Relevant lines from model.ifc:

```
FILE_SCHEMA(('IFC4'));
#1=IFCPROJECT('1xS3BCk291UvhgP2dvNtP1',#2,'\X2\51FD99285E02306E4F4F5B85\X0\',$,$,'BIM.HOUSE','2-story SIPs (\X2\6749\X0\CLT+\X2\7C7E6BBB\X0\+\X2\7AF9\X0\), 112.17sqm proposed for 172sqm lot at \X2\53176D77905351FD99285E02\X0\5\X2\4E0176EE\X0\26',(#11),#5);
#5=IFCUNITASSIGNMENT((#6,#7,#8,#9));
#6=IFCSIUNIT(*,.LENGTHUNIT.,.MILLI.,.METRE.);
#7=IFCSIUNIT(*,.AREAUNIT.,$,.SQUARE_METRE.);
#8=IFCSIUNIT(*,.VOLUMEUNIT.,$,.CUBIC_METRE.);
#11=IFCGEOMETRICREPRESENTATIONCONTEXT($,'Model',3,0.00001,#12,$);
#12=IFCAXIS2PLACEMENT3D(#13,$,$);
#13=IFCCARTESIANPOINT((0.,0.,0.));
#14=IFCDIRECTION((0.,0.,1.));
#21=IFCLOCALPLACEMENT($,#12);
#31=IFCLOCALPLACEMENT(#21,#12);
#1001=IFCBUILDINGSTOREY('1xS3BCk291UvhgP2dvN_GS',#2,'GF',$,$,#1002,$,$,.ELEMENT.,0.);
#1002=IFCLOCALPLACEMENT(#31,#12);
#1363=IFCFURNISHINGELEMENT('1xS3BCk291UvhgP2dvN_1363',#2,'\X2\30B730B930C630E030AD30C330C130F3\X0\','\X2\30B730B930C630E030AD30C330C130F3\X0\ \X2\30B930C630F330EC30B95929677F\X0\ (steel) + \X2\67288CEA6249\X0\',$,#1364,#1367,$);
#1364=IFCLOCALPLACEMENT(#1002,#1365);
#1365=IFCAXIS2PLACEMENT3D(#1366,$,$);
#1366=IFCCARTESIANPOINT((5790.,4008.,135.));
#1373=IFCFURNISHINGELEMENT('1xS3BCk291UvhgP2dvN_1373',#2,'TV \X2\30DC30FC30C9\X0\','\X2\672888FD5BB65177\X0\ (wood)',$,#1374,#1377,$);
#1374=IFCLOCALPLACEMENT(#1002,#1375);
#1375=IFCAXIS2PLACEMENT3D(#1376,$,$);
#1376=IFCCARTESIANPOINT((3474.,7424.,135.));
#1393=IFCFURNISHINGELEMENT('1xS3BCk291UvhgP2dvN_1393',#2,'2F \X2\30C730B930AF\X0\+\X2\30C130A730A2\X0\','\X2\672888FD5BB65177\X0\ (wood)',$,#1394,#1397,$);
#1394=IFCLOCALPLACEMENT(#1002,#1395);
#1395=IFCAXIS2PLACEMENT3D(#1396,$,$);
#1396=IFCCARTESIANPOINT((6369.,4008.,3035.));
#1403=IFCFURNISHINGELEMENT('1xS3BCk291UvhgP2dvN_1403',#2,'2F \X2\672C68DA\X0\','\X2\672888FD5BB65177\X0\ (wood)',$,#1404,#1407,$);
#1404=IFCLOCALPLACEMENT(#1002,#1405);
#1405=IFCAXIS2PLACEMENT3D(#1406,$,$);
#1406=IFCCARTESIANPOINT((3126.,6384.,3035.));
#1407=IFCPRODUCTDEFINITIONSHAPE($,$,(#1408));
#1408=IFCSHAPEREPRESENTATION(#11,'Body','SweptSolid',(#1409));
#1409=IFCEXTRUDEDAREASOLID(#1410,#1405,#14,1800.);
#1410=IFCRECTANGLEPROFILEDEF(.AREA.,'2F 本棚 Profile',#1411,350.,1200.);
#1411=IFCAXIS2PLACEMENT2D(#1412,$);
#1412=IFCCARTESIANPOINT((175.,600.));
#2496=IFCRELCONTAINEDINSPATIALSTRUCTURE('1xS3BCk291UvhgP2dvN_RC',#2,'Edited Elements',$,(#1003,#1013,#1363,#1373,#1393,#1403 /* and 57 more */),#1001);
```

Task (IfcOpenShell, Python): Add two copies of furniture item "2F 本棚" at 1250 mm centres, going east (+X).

```python
import numpy as np
import ifcopenshell
import ifcopenshell.api.geometry
import ifcopenshell.api.root
import ifcopenshell.util.element
import ifcopenshell.util.placement
import ifcopenshell.util.unit

model = ifcopenshell.open("model.ifc")
unit_scale = ifcopenshell.util.unit.calculate_unit_scale(model)


def reuse_history(source, copy):
    """copy_class also copies each property set's owner history, people and application; keep the originals."""
    for rel in copy.IsDefinedBy:
        if rel.is_a("IfcRelDefinesByProperties") and (history := rel.RelatingPropertyDefinition.OwnerHistory):
            rel.RelatingPropertyDefinition.OwnerHistory = source.OwnerHistory
            ifcopenshell.util.element.remove_deep2(model, history)


source = model.by_id(1403)
base = ifcopenshell.util.placement.get_local_placement(source.ObjectPlacement)
step = np.array([1.0, 0.0, 0.0]) * 1.25 / unit_scale

for i in range(1, 3):
    copy = ifcopenshell.api.root.copy_class(model, product=source)
    copy.Representation = ifcopenshell.util.element.copy_deep(
        model, source.Representation, exclude=["IfcGeometricRepresentationContext", "IfcRepresentationMap"]
    )
    reuse_history(source, copy)
    matrix = base.copy()
    matrix[:3, 3] += i * step
    print("added at", matrix[:3, 3].round(3) + 0.0)
    ifcopenshell.api.geometry.edit_object_placement(model, product=copy, matrix=matrix, is_si=False)

model.write("model_v2.ifc")
```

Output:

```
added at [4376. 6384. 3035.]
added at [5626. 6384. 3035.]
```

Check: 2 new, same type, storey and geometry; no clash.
